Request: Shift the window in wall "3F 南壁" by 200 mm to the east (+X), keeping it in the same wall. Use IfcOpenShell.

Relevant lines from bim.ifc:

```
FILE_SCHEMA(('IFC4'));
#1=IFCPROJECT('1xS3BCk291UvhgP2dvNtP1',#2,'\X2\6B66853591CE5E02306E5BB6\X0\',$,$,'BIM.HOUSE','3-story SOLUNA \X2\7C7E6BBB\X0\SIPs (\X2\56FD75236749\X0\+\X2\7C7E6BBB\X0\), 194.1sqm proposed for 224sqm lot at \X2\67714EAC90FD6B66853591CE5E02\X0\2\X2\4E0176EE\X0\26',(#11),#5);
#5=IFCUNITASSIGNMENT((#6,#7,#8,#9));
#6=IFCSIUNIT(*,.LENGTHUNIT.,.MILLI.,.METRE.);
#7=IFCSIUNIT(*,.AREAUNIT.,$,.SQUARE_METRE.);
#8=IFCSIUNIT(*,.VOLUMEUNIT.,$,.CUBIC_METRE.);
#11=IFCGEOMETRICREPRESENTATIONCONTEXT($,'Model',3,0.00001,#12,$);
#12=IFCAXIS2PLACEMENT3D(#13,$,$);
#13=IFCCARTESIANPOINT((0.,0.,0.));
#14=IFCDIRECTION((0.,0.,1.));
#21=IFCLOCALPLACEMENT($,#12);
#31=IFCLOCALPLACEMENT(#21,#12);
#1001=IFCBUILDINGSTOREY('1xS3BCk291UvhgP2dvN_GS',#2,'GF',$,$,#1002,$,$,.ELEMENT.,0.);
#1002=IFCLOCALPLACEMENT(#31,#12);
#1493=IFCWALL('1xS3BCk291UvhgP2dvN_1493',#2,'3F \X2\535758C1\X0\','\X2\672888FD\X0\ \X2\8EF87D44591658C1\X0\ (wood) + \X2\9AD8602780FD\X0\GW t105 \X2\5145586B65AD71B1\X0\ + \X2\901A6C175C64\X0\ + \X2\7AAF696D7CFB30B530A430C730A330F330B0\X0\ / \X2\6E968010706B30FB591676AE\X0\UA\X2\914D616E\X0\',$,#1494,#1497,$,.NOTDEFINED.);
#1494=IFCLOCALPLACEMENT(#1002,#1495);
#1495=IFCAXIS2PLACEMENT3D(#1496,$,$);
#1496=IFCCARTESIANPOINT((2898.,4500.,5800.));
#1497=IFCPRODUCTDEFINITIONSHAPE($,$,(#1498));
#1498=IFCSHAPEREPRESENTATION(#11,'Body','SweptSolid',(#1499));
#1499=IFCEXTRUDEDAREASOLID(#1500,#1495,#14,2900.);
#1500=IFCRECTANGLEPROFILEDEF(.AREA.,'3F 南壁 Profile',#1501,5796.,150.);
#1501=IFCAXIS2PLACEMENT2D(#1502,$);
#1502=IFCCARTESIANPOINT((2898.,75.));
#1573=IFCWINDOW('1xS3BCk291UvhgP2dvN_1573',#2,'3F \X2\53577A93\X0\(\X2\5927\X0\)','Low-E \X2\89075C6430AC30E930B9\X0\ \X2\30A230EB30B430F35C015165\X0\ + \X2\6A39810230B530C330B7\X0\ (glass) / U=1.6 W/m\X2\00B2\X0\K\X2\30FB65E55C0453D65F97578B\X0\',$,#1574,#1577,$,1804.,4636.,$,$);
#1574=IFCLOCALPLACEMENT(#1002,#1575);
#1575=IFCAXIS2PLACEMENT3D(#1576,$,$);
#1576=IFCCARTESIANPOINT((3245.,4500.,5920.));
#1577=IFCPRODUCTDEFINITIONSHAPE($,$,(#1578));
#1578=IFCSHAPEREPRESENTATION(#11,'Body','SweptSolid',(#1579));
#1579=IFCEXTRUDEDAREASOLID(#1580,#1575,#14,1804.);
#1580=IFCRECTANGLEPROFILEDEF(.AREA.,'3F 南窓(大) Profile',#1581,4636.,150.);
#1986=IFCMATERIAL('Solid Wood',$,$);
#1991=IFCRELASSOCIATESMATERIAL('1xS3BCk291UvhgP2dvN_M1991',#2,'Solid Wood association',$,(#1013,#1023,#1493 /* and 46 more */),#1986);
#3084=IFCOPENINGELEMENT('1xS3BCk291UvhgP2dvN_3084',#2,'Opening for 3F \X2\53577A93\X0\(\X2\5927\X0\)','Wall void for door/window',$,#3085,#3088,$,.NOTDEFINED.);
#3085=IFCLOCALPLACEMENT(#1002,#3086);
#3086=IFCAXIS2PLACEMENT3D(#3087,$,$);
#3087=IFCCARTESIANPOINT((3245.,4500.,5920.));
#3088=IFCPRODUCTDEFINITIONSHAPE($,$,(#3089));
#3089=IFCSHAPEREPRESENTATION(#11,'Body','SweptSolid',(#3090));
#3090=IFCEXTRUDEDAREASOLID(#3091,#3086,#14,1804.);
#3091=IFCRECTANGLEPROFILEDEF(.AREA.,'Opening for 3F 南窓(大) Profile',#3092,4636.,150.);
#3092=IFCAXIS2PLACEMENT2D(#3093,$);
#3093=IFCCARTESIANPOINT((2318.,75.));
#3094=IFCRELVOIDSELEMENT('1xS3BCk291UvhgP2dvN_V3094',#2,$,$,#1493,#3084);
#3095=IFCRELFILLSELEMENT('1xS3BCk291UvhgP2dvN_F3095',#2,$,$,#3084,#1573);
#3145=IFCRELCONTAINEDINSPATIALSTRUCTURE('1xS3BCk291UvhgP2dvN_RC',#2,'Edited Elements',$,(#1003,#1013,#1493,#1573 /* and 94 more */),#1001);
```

```python
import ifcopenshell
import ifcopenshell.api.geometry
import ifcopenshell.util.placement

model = ifcopenshell.open("bim.ifc")

window = model.by_guid("1xS3BCk291UvhgP2dvN_1573")
opening = window.FillsVoids[0].RelatingOpeningElement
wall = opening.VoidsElements[0].RelatingBuildingElement

wall_matrix = ifcopenshell.util.placement.get_local_placement(wall.ObjectPlacement)
shift = wall_matrix[:3, 0] * 200.0
before = ifcopenshell.util.placement.get_local_placement(window.ObjectPlacement)[:3, 3].copy()

# The window is not placed relative to its opening, so move both.
for product in (opening, window):
    matrix = ifcopenshell.util.placement.get_local_placement(product.ObjectPlacement)
    matrix[:3, 3] += shift
    ifcopenshell.api.geometry.edit_object_placement(model, product=product, matrix=matrix, is_si=False)

after = ifcopenshell.util.placement.get_local_placement(window.ObjectPlacement)[:3, 3]
print("window moved by", (after - before).round(3) + 0.0)

model.write("bim_updated.ifc")
```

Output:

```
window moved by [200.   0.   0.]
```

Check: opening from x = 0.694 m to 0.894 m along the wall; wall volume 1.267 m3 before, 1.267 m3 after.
